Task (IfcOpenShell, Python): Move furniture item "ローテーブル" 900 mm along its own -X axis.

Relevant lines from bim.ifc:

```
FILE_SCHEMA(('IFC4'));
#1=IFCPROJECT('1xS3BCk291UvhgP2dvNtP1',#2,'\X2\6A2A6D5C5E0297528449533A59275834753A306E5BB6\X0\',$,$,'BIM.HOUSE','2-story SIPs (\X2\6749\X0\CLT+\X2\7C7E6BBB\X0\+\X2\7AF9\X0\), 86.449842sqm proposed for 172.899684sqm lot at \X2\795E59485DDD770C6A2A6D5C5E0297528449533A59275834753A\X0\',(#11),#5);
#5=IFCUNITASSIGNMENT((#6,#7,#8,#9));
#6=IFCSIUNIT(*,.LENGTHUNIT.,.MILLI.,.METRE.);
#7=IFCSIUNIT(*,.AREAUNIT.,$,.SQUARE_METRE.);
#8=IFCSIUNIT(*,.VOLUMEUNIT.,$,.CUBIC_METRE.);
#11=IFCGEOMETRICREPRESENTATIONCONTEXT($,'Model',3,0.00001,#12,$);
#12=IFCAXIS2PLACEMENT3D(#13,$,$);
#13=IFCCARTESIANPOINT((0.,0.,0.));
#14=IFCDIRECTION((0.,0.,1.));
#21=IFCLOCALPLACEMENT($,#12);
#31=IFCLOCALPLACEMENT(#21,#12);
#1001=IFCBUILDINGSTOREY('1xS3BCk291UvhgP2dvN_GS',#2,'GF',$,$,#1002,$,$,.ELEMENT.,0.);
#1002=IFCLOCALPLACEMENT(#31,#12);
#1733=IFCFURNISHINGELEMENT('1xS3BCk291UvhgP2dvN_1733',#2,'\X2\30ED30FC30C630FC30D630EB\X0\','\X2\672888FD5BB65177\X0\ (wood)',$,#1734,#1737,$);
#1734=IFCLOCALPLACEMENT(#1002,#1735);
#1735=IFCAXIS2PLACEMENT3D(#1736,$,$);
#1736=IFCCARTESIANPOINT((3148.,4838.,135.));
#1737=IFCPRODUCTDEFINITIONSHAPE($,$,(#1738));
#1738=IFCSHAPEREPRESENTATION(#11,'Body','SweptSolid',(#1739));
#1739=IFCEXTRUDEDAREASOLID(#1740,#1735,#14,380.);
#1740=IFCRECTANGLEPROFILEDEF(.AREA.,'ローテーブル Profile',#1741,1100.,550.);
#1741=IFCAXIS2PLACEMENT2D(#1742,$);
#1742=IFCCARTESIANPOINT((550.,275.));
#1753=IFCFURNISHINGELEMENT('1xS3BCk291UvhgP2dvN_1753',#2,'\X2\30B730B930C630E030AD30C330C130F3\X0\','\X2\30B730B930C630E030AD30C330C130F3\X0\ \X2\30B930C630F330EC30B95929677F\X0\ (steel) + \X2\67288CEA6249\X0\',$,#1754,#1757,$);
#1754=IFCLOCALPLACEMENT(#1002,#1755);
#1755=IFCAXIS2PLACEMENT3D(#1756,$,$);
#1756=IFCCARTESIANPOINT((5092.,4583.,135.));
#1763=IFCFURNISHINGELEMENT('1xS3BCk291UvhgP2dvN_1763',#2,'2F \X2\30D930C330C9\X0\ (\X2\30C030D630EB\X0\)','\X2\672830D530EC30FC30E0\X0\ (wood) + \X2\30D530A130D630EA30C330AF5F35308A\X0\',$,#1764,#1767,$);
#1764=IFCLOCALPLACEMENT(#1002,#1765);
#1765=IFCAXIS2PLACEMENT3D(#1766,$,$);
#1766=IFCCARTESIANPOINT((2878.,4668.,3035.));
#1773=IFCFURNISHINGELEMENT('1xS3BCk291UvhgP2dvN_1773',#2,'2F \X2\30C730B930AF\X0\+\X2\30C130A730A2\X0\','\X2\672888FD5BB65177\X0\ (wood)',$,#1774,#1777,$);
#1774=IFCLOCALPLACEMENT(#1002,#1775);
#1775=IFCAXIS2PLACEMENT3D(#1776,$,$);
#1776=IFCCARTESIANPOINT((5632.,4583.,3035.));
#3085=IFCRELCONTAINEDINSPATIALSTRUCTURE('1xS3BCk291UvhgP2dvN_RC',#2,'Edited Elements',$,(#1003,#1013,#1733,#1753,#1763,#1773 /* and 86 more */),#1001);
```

```python
import ifcopenshell
import ifcopenshell.api.geometry
import ifcopenshell.util.placement
import ifcopenshell.util.unit

model = ifcopenshell.open("bim.ifc")
unit_scale = ifcopenshell.util.unit.calculate_unit_scale(model)

item = model.by_id(1733)
matrix = ifcopenshell.util.placement.get_local_placement(item.ObjectPlacement)
matrix[:3, 3] -= matrix[:3, 0] * 0.9 / unit_scale
ifcopenshell.api.geometry.edit_object_placement(model, product=item, matrix=matrix, is_si=False)

print(ifcopenshell.util.placement.get_local_placement(item.ObjectPlacement).round(3) + 0.0)

model.write("bim_updated.ifc")
```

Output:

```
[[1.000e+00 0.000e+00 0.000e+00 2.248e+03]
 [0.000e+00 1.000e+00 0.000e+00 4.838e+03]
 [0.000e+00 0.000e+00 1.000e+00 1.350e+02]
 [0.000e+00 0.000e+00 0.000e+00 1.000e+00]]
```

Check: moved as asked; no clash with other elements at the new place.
